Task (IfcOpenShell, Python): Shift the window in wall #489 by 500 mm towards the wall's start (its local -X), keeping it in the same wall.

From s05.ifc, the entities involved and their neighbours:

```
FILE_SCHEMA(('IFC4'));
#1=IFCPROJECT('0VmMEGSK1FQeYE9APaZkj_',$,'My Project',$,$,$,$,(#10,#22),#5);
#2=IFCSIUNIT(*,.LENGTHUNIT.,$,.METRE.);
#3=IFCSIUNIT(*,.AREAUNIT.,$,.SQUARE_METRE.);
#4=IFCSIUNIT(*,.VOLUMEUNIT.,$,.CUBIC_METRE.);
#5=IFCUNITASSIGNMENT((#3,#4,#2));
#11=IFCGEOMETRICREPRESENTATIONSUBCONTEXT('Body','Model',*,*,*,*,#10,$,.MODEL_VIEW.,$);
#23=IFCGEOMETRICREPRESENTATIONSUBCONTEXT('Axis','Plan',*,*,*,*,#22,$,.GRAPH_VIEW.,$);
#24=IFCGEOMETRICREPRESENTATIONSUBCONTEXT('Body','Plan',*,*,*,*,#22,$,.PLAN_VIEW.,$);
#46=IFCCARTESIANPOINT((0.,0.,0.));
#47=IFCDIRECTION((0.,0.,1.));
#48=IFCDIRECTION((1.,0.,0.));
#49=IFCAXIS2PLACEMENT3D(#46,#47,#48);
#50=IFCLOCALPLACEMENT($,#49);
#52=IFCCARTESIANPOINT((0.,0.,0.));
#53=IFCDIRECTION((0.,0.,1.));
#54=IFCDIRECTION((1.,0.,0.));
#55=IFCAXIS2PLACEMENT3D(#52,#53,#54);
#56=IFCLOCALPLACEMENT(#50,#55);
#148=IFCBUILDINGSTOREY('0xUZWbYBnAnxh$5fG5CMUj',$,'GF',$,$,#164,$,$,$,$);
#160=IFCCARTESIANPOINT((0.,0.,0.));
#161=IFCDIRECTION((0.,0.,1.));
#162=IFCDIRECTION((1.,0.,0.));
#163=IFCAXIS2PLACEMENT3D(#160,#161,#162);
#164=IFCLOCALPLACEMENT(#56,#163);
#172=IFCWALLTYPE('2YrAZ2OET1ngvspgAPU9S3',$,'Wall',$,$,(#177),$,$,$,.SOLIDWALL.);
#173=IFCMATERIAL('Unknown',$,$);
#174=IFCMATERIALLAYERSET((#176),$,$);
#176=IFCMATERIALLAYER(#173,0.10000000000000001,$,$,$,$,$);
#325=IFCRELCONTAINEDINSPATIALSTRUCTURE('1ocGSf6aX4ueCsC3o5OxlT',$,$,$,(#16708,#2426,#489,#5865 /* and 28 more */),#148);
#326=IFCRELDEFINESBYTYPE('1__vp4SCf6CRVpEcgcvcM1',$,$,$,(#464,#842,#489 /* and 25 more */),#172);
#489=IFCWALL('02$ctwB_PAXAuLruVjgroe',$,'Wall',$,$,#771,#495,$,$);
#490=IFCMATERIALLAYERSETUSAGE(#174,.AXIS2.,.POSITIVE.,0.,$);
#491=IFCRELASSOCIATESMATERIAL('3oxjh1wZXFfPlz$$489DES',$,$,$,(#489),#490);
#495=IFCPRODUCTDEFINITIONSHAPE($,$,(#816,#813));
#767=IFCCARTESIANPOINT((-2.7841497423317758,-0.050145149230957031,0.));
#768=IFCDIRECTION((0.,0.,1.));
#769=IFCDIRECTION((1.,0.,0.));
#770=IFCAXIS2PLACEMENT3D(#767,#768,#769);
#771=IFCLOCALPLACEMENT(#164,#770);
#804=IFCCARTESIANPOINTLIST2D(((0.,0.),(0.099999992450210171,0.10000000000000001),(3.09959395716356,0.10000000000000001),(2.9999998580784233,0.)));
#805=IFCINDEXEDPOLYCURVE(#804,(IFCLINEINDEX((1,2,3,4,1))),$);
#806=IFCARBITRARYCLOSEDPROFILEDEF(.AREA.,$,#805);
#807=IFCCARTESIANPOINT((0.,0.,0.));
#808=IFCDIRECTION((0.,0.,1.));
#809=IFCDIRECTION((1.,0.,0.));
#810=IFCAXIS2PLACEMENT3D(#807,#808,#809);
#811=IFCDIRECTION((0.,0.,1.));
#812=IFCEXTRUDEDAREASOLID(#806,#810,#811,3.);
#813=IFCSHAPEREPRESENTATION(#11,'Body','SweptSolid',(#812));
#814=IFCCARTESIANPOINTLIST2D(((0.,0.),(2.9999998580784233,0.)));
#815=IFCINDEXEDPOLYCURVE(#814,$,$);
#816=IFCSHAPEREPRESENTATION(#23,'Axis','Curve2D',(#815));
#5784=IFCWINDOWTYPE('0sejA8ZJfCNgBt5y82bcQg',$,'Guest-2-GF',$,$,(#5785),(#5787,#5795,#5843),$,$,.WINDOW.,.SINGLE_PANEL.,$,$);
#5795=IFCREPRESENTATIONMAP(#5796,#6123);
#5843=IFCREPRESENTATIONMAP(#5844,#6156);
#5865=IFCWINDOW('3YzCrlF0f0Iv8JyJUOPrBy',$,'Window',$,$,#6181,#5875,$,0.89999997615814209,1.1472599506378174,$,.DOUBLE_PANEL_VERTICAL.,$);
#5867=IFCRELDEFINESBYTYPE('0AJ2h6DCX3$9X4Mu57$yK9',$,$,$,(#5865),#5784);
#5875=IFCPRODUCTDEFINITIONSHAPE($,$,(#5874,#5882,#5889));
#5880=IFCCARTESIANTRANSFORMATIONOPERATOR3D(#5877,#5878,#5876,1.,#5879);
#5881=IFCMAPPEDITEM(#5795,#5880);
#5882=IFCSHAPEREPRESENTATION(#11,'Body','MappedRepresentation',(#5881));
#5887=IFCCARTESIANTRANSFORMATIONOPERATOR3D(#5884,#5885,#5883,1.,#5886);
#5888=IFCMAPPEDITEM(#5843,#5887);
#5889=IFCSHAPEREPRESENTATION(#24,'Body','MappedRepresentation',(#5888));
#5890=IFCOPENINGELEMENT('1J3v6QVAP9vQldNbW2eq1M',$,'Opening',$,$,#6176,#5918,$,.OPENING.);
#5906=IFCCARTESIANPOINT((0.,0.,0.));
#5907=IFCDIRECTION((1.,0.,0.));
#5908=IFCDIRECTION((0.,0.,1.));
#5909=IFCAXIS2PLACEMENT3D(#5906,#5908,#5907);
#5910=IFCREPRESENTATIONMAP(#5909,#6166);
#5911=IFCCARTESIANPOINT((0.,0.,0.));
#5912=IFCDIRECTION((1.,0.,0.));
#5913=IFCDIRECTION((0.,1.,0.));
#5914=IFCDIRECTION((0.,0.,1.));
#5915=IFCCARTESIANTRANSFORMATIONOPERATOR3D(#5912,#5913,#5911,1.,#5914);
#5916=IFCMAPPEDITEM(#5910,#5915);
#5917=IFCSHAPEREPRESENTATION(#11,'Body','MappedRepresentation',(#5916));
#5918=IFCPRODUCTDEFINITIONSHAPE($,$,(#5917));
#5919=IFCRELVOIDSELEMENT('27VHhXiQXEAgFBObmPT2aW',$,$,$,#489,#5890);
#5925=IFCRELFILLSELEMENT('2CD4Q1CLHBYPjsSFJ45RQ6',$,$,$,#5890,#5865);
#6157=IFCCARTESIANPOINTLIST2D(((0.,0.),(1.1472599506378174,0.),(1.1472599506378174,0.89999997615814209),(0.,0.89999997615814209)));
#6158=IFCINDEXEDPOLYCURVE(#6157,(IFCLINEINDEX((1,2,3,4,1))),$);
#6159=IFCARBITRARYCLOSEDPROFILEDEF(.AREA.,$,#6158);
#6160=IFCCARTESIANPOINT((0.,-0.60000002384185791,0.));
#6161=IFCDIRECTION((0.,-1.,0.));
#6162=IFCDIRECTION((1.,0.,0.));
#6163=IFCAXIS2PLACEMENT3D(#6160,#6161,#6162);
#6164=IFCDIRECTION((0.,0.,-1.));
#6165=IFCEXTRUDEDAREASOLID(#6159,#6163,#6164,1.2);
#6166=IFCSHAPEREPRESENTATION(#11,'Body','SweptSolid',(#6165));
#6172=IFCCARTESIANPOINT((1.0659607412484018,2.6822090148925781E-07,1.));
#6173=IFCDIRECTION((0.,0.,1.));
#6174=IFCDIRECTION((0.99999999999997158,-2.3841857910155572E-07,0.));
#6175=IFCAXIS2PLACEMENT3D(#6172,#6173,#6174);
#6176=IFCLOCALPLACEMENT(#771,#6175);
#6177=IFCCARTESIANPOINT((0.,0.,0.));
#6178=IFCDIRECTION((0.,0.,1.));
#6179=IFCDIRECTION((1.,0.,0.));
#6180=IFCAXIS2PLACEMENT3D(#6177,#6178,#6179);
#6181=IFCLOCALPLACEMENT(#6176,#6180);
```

```python
import ifcopenshell
import ifcopenshell.api.geometry
import ifcopenshell.util.placement
import ifcopenshell.util.unit

model = ifcopenshell.open("s05.ifc")
unit_scale = ifcopenshell.util.unit.calculate_unit_scale(model)

window = model.by_id(5865)
opening = window.FillsVoids[0].RelatingOpeningElement
wall = opening.VoidsElements[0].RelatingBuildingElement

wall_matrix = ifcopenshell.util.placement.get_local_placement(wall.ObjectPlacement)
shift = wall_matrix[:3, 0] * -0.5 / unit_scale
before = ifcopenshell.util.placement.get_local_placement(window.ObjectPlacement)[:3, 3].copy()

# The window is placed relative to its opening, so it follows when the opening moves.
matrix = ifcopenshell.util.placement.get_local_placement(opening.ObjectPlacement)
matrix[:3, 3] += shift
ifcopenshell.api.geometry.edit_object_placement(
    model, product=opening, matrix=matrix, is_si=False, should_transform_children=True
)

after = ifcopenshell.util.placement.get_local_placement(window.ObjectPlacement)[:3, 3]
print("window moved by", (after - before).round(3) + 0.0)

model.write("s05_updated.ifc")
```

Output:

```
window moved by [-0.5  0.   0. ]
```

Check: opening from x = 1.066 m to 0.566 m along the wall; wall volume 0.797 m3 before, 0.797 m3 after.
